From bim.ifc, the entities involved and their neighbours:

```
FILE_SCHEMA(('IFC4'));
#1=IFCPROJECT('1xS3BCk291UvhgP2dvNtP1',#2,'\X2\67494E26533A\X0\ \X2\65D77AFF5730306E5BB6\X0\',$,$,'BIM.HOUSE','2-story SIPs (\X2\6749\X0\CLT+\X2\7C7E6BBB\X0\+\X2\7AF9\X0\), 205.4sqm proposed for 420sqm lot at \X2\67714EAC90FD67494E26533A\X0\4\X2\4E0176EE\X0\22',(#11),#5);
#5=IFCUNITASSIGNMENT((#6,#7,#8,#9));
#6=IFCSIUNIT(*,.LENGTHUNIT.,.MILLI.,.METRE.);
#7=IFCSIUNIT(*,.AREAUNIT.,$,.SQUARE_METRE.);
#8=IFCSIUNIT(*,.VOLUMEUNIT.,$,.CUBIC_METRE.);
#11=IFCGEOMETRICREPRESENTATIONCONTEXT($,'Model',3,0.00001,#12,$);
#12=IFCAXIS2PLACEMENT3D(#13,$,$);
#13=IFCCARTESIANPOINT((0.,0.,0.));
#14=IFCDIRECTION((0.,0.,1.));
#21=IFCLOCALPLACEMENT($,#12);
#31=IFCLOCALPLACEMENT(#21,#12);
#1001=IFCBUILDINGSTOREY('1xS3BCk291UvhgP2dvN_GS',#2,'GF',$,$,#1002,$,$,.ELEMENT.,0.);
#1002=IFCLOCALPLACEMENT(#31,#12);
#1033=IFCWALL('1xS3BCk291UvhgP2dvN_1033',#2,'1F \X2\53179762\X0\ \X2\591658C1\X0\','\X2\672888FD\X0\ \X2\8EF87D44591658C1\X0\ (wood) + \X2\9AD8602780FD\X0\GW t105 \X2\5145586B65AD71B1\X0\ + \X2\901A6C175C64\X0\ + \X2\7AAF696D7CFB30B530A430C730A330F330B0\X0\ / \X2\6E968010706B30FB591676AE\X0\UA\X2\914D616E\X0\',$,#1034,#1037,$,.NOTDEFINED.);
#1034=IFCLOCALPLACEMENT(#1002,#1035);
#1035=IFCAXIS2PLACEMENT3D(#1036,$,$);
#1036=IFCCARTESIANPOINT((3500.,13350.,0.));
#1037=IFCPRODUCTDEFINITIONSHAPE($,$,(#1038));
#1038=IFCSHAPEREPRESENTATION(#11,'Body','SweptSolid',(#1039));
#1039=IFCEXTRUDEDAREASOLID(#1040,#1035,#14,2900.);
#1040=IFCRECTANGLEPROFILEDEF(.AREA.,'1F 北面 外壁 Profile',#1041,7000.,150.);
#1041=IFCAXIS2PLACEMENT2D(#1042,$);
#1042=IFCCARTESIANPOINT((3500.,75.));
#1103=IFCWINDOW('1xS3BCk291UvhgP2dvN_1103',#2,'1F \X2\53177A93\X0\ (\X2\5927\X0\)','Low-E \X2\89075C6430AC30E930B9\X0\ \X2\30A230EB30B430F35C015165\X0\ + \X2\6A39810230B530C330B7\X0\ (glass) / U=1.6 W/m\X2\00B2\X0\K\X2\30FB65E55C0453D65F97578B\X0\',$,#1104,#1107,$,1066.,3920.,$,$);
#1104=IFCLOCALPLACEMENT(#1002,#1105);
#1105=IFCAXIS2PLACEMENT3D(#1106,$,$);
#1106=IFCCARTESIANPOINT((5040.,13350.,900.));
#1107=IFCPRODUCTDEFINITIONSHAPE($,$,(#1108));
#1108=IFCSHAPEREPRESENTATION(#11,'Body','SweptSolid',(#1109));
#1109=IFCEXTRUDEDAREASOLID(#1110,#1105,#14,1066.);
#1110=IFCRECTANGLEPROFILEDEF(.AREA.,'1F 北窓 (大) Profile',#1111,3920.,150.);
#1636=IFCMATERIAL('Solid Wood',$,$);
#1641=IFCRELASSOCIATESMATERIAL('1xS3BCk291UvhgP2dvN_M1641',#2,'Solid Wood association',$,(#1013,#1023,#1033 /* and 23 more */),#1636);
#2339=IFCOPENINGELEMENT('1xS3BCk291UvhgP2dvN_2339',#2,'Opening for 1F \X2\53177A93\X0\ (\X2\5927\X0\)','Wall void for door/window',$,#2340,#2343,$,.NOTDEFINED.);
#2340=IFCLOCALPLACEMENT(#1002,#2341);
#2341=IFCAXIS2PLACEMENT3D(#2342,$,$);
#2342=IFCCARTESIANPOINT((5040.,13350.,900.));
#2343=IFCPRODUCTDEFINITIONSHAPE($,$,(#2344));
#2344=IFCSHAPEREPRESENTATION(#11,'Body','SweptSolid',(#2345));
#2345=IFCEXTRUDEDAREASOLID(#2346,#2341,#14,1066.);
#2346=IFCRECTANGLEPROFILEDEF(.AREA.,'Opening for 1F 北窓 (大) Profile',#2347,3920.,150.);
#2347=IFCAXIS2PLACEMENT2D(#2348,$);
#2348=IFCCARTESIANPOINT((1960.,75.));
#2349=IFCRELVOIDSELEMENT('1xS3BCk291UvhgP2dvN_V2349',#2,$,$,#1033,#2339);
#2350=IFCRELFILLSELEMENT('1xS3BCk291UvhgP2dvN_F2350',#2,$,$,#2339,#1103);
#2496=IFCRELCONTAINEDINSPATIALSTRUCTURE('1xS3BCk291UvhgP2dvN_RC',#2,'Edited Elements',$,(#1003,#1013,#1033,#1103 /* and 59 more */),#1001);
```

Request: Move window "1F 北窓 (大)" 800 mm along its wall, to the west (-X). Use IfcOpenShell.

```python
import ifcopenshell
import ifcopenshell.api.geometry
import ifcopenshell.util.placement

model = ifcopenshell.open("bim.ifc")

window = model.by_guid("1xS3BCk291UvhgP2dvN_1103")
opening = window.FillsVoids[0].RelatingOpeningElement
wall = opening.VoidsElements[0].RelatingBuildingElement

wall_matrix = ifcopenshell.util.placement.get_local_placement(wall.ObjectPlacement)
shift = wall_matrix[:3, 0] * -800.0
before = ifcopenshell.util.placement.get_local_placement(window.ObjectPlacement)[:3, 3].copy()

# The window is not placed relative to its opening, so move both.
for product in (opening, window):
    matrix = ifcopenshell.util.placement.get_local_placement(product.ObjectPlacement)
    matrix[:3, 3] += shift
    ifcopenshell.api.geometry.edit_object_placement(model, product=product, matrix=matrix, is_si=False)

after = ifcopenshell.util.placement.get_local_placement(window.ObjectPlacement)[:3, 3]
print("window moved by", (after - before).round(3) + 0.0)

model.write("bim-out.ifc")
```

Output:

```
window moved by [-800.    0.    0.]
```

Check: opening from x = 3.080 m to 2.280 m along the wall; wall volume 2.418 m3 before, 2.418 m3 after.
